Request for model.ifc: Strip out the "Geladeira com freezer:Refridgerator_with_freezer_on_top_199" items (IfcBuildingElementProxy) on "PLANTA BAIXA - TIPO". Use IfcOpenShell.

First a look at what the model holds.

```python
import ifcopenshell
import ifcopenshell.util.element

model = ifcopenshell.open("model.ifc")
print(model.schema)
storey = next(s for s in model.by_type("IfcBuildingStorey") if s.Name == "PLANTA BAIXA - TIPO")
proxies = [e for e in ifcopenshell.util.element.get_decomposition(storey) if e.is_a("IfcBuildingElementProxy")]
seen = {}
for e in proxies:
    element_type = ifcopenshell.util.element.get_type(e)
    name = element_type.Name if element_type not in (None, e) else None
    seen[name] = seen.get(name, 0) + 1
for name, count in sorted(seen.items(), key=str):
    print(count, "x", name)
```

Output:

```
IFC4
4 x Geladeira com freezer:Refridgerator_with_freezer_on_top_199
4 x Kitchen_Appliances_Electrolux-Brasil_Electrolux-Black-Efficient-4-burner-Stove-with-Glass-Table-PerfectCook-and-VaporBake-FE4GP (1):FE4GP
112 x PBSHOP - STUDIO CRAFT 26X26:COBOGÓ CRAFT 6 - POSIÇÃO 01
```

```python
import ifcopenshell
import ifcopenshell.api.root
import ifcopenshell.util.element

model = ifcopenshell.open("model.ifc")

storey = next(s for s in model.by_type("IfcBuildingStorey") if s.Name == "PLANTA BAIXA - TIPO")
proxies = [e for e in ifcopenshell.util.element.get_decomposition(storey) if e.is_a("IfcBuildingElementProxy")]
targets = [e for e in proxies if (t := ifcopenshell.util.element.get_type(e)) not in (None, e) and t.Name == "Geladeira com freezer:Refridgerator_with_freezer_on_top_199"]

for e in targets:
    ifcopenshell.api.root.remove_product(model, product=e)
print(len(targets), "removed")

model.write("model_edited.ifc")
```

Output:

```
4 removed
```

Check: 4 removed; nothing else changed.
